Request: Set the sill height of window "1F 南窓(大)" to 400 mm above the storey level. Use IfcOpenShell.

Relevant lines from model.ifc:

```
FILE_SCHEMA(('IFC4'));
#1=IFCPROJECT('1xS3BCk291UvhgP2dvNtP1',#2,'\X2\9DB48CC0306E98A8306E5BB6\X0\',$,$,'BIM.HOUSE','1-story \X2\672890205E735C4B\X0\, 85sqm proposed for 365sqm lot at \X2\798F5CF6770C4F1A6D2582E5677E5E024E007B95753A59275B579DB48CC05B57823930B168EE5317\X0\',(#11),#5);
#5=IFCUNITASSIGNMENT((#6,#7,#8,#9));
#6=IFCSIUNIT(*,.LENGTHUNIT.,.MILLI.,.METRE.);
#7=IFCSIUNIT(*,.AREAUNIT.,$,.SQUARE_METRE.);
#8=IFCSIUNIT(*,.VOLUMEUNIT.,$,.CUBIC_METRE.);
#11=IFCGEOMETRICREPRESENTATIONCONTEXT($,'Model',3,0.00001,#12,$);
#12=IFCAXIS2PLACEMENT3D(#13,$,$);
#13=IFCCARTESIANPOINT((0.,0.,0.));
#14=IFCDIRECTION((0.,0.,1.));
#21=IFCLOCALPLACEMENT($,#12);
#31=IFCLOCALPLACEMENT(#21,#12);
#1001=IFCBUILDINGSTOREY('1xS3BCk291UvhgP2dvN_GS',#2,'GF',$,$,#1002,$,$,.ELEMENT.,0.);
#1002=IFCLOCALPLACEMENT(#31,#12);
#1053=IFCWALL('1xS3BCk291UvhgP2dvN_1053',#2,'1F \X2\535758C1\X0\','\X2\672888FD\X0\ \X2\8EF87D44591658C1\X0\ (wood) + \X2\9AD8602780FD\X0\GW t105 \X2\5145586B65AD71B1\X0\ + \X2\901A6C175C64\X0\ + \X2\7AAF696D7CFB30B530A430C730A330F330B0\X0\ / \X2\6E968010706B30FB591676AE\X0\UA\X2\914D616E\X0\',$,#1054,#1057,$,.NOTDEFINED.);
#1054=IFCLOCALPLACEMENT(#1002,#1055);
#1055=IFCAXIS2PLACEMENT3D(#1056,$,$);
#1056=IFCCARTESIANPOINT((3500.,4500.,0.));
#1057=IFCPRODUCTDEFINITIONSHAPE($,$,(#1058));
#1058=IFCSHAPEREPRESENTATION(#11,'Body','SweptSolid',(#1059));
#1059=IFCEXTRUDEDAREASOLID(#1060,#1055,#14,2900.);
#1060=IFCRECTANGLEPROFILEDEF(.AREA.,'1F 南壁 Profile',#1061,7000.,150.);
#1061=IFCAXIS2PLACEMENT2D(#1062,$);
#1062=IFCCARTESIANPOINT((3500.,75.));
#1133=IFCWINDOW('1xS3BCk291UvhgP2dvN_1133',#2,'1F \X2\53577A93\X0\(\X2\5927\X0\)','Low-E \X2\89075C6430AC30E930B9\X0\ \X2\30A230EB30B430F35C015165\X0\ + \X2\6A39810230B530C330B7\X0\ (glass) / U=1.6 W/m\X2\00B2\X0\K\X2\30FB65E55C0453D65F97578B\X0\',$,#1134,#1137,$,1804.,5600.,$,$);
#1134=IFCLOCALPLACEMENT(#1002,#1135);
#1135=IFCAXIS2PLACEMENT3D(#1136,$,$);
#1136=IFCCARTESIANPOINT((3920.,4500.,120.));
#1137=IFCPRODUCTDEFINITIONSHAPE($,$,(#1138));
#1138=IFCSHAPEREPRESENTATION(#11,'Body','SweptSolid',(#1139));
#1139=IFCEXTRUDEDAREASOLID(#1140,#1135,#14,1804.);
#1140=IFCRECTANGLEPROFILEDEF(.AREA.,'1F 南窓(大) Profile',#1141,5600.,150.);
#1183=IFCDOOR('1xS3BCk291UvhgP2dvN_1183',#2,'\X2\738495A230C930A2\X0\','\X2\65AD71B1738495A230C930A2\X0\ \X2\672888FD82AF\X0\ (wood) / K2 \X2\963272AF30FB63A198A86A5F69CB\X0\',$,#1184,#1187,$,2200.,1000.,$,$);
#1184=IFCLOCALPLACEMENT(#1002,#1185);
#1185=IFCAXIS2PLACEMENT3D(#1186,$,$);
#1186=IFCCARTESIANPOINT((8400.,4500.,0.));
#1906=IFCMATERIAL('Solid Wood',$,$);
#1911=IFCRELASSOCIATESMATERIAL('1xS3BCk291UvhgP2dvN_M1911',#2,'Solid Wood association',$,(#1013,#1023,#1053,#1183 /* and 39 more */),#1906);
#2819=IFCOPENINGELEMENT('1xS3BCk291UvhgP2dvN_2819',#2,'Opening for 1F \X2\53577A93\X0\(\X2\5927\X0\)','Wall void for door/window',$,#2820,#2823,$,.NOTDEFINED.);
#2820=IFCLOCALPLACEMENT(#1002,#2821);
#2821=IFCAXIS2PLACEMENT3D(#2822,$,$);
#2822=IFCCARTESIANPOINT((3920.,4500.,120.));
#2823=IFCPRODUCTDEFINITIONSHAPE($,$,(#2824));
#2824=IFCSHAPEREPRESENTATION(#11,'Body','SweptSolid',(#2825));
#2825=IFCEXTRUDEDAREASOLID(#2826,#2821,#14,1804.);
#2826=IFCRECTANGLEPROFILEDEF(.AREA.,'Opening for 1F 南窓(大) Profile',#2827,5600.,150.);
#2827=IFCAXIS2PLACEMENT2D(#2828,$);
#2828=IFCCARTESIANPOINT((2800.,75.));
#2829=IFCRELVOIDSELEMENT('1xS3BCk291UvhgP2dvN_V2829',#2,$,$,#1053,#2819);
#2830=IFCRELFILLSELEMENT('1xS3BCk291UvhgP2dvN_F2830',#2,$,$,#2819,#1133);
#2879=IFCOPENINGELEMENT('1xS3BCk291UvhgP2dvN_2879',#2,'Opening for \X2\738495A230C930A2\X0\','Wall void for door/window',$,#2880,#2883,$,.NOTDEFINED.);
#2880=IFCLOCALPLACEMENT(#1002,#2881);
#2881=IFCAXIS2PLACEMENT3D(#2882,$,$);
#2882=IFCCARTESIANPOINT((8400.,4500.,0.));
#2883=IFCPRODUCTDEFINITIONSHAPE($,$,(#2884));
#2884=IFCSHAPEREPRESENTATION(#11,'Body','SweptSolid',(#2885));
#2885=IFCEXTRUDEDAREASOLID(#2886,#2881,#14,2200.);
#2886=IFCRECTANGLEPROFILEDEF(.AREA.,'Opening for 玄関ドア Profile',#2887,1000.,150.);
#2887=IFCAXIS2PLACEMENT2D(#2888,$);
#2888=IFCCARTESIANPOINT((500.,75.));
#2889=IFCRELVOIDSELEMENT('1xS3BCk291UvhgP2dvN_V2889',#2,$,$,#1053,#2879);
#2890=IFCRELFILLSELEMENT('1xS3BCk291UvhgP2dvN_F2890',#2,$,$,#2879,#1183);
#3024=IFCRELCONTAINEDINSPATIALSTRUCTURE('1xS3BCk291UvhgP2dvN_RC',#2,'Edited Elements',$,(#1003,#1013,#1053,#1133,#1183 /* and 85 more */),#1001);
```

```python
import numpy as np
import ifcopenshell
import ifcopenshell.api.geometry
import ifcopenshell.geom
import ifcopenshell.util.element
import ifcopenshell.util.placement
import ifcopenshell.util.shape
import ifcopenshell.util.unit

model = ifcopenshell.open("model.ifc")
unit_scale = ifcopenshell.util.unit.calculate_unit_scale(model)

window = model.by_guid("1xS3BCk291UvhgP2dvN_1133")
opening = window.FillsVoids[0].RelatingOpeningElement
storey = ifcopenshell.util.element.get_container(window, ifc_class="IfcBuildingStorey")
level = ifcopenshell.util.placement.get_local_placement(storey.ObjectPlacement)[2, 3]

# The opening's origin need not be at the sill, so measure its lowest point.
shape = ifcopenshell.geom.create_shape(ifcopenshell.geom.settings(), opening)
bottom = ifcopenshell.util.shape.get_shape_bottom_elevation(shape, shape.geometry) / unit_scale
dz = level + 400.0 - bottom

shift = np.array([0.0, 0.0, dz])
# The window is not placed relative to its opening, so move both.
for product in (opening, window):
    matrix = ifcopenshell.util.placement.get_local_placement(product.ObjectPlacement)
    matrix[:3, 3] += shift
    ifcopenshell.api.geometry.edit_object_placement(model, product=product, matrix=matrix, is_si=False)

print(f"moved by {dz * unit_scale:+.3f} m")

model.write("model_rev.ifc")
```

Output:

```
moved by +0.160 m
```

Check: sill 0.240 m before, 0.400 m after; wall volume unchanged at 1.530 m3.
